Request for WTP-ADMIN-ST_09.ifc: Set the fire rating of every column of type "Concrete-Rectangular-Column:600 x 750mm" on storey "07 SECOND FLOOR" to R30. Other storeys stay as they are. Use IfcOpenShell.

First a look at what the model holds.

```python
import ifcopenshell
import ifcopenshell.util.element

model = ifcopenshell.open("WTP-ADMIN-ST_09.ifc")
print(model.schema)
storey = next(s for s in model.by_type("IfcBuildingStorey") if s.Name == "07 SECOND FLOOR")
columns = [e for e in ifcopenshell.util.element.get_decomposition(storey) if e.is_a("IfcColumn")]
seen = {}
for e in columns:
    element_type = ifcopenshell.util.element.get_type(e)
    key = (element_type.Name if element_type != e and element_type else None, ifcopenshell.util.element.get_pset(e, "Pset_ColumnCommon", "FireRating"))
    seen[key] = seen.get(key, 0) + 1
for (name, value), count in sorted(seen.items(), key=str):
    print(count, "x", name, "|", value)
```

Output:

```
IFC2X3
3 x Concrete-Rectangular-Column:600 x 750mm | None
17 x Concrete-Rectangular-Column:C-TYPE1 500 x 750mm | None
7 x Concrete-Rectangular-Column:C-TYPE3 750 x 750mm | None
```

```python
import ifcopenshell
import ifcopenshell.api.pset
import ifcopenshell.util.element

model = ifcopenshell.open("WTP-ADMIN-ST_09.ifc")

storey = next(s for s in model.by_type("IfcBuildingStorey") if s.Name == "07 SECOND FLOOR")
columns = [e for e in ifcopenshell.util.element.get_decomposition(storey) if e.is_a("IfcColumn")]

count = 0
for e in columns:
    element_type = ifcopenshell.util.element.get_type(e)
    if element_type in (None, e) or element_type.Name != "Concrete-Rectangular-Column:600 x 750mm":
        continue
    # add_pset returns the element's existing set when there is one.
    pset = ifcopenshell.api.pset.add_pset(model, product=e, name="Pset_ColumnCommon")
    ifcopenshell.api.pset.edit_pset(model, pset=pset, properties={"FireRating": "R30"})
    count += 1

print(count, "columns updated")

model.write("WTP-ADMIN-ST_09_v2.ifc")
```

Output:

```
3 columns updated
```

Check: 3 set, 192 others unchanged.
